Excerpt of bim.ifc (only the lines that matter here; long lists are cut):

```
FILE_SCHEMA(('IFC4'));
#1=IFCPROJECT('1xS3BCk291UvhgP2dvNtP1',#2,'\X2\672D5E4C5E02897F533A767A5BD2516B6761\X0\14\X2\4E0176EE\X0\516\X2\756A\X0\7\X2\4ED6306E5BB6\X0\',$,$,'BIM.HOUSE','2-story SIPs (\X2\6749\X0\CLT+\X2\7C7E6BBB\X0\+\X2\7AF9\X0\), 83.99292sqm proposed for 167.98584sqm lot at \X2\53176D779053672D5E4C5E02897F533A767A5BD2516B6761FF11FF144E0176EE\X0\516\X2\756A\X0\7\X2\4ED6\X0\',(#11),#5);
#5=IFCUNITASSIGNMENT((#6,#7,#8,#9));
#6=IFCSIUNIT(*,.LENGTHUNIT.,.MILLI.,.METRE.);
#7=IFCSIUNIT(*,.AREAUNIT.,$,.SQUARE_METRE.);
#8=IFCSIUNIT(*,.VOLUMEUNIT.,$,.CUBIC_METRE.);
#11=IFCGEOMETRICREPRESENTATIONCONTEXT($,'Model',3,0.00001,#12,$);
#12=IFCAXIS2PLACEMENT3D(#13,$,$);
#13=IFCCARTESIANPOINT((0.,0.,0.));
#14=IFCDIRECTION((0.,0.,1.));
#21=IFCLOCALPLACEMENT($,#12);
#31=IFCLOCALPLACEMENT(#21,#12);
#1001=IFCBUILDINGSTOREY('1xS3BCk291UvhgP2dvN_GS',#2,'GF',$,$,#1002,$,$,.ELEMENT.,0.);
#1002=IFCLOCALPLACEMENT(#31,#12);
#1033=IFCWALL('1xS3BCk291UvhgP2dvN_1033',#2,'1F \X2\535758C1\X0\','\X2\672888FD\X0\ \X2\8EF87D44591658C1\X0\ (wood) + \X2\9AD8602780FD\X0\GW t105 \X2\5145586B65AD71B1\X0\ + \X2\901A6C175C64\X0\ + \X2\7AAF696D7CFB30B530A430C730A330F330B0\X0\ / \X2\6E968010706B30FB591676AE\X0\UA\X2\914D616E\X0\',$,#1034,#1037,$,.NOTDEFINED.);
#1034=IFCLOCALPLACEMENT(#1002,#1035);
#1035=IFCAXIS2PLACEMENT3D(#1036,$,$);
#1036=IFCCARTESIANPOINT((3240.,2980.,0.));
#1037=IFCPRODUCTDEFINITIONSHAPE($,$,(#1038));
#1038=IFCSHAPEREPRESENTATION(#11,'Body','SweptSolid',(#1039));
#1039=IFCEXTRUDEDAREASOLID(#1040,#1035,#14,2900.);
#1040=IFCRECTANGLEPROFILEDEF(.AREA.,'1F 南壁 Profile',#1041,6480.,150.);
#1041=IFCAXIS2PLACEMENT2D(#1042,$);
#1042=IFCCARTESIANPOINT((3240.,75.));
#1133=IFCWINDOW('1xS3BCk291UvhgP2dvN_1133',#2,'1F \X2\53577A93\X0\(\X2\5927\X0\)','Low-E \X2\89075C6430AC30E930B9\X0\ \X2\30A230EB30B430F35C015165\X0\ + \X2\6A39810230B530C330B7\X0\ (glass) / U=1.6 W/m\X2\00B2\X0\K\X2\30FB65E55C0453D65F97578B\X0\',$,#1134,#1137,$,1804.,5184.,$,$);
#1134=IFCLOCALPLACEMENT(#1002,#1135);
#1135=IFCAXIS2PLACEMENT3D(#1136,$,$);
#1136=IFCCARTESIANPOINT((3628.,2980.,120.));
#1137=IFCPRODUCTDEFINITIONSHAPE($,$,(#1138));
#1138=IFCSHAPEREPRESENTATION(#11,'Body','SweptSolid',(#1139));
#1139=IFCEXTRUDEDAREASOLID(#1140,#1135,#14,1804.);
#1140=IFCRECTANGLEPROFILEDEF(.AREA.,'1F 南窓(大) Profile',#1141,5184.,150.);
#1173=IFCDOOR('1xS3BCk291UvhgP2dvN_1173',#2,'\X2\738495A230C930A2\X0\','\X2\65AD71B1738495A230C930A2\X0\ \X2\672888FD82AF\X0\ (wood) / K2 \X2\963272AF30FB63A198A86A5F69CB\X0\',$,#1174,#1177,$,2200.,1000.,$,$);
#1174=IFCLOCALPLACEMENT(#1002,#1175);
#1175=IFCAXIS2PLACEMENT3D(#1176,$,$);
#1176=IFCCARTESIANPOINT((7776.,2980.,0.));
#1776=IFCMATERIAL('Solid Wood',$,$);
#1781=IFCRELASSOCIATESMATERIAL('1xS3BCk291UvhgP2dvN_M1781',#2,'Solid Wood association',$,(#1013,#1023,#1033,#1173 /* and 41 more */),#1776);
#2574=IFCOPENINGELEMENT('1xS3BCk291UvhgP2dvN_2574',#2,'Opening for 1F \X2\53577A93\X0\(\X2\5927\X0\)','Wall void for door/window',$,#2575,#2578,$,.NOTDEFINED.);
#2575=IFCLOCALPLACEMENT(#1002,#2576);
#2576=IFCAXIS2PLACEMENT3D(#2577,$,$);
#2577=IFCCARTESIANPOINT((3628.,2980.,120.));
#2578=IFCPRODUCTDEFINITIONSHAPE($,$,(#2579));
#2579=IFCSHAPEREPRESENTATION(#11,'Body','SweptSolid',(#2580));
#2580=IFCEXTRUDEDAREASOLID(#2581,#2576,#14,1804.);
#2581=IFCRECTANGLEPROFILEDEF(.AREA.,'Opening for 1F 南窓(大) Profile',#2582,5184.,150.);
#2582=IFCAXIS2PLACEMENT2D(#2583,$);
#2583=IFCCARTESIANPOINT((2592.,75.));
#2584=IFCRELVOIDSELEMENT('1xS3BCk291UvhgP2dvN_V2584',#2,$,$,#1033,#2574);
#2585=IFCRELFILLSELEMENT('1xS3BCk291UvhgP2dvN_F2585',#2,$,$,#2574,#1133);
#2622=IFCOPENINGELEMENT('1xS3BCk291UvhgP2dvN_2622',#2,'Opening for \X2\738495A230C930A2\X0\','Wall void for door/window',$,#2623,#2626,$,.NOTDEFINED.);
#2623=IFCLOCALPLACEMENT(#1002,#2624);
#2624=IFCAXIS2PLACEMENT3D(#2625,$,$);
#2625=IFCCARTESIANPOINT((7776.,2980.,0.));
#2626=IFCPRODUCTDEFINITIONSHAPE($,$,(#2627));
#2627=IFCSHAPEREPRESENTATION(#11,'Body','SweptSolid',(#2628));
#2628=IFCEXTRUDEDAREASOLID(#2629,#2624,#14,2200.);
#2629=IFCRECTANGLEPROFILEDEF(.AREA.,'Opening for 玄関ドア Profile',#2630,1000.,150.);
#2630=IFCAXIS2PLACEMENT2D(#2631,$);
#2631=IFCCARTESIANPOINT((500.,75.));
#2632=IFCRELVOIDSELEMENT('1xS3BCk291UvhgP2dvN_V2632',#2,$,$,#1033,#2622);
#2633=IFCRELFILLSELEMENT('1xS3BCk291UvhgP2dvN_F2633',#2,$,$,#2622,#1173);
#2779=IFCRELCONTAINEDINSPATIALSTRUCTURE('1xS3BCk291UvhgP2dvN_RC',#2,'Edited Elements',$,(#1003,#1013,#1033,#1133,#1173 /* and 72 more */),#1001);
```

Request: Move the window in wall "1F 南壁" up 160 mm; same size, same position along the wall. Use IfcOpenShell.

```python
import numpy as np
import ifcopenshell
import ifcopenshell.api.geometry
import ifcopenshell.util.placement
import ifcopenshell.util.unit

model = ifcopenshell.open("bim.ifc")
unit_scale = ifcopenshell.util.unit.calculate_unit_scale(model)

window = model.by_guid("1xS3BCk291UvhgP2dvN_1133")
opening = window.FillsVoids[0].RelatingOpeningElement
dz = 160.0

shift = np.array([0.0, 0.0, dz])
# The window is not placed relative to its opening, so move both.
for product in (opening, window):
    matrix = ifcopenshell.util.placement.get_local_placement(product.ObjectPlacement)
    matrix[:3, 3] += shift
    ifcopenshell.api.geometry.edit_object_placement(model, product=product, matrix=matrix, is_si=False)

print(f"moved by {dz * unit_scale:+.3f} m")

model.write("bim-out.ifc")
```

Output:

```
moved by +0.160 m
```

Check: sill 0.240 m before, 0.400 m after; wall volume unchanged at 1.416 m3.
